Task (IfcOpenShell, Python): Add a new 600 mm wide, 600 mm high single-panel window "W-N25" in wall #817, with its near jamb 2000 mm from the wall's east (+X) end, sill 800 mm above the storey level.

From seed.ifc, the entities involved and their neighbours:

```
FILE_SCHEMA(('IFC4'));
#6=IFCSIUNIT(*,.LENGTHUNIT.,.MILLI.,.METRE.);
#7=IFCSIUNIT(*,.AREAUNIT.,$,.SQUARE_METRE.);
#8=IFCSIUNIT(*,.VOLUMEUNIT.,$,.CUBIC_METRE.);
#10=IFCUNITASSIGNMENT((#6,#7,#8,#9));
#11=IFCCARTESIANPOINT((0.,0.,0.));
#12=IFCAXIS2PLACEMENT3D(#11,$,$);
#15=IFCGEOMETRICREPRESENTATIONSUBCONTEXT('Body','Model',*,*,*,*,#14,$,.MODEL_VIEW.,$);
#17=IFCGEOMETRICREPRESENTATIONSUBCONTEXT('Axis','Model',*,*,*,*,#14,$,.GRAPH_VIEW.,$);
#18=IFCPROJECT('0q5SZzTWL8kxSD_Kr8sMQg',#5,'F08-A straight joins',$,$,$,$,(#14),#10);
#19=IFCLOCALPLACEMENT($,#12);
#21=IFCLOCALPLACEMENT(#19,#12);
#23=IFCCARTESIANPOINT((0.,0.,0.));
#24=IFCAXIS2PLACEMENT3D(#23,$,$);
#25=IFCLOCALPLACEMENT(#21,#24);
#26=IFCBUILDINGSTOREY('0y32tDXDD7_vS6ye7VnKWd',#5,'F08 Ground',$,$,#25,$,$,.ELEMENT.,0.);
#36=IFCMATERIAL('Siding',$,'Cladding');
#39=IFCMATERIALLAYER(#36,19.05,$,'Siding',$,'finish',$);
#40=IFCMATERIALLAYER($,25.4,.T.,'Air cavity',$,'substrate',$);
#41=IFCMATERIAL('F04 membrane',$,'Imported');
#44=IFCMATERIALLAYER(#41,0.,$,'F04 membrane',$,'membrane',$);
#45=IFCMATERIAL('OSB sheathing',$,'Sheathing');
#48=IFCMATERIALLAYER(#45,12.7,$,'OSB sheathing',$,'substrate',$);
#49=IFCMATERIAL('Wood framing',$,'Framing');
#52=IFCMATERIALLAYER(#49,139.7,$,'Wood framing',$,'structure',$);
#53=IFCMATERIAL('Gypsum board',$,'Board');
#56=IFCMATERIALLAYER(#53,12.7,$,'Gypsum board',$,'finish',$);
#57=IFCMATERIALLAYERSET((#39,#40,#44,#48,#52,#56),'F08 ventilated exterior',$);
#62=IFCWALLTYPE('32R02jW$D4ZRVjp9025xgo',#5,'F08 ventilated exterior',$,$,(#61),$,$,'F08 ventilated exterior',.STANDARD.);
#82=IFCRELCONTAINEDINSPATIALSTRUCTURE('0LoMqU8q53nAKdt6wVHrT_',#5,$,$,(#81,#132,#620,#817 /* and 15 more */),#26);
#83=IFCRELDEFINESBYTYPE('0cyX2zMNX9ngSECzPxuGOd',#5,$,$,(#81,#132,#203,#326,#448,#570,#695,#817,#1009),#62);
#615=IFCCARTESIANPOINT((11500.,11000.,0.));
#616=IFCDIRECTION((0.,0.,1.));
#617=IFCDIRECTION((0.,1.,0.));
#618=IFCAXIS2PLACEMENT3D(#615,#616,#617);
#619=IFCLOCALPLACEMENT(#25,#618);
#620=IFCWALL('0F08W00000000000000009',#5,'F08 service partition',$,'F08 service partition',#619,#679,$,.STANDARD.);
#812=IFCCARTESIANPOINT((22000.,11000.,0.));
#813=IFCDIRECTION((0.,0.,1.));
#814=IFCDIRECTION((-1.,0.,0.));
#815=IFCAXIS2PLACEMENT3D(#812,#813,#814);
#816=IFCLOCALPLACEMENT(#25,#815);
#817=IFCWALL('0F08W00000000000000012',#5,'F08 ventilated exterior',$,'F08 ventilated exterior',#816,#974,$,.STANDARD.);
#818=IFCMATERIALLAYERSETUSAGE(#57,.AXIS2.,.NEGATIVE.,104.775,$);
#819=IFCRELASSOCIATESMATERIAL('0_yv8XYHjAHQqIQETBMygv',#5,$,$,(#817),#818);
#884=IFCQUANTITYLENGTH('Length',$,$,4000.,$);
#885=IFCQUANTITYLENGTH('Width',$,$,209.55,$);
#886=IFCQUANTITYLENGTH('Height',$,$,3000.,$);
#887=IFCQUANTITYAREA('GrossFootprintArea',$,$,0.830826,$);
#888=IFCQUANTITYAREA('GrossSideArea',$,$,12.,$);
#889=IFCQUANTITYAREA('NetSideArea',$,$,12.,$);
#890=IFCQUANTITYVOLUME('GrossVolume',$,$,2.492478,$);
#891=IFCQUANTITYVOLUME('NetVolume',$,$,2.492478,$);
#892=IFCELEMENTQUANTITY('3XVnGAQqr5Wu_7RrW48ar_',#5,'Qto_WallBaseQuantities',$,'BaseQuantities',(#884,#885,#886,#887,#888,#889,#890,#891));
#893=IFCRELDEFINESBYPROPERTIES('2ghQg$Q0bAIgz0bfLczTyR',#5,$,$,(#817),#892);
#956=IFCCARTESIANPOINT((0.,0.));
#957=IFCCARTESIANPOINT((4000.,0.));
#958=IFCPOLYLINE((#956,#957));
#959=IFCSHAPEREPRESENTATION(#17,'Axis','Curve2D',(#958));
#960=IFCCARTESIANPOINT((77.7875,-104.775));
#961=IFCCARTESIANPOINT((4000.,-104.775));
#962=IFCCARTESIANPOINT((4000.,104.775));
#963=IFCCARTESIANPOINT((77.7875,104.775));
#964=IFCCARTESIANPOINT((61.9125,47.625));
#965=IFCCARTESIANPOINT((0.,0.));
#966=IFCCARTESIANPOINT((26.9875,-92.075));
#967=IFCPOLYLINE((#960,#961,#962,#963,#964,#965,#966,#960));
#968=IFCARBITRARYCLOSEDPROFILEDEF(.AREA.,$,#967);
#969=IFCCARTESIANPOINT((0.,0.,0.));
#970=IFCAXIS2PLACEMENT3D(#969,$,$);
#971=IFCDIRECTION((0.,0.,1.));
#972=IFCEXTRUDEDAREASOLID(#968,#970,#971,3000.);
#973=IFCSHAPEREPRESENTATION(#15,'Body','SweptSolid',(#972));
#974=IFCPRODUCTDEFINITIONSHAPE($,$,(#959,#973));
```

```python
import numpy as np
import ifcopenshell
import ifcopenshell.api.feature
import ifcopenshell.api.geometry
import ifcopenshell.api.pset
import ifcopenshell.api.root
import ifcopenshell.api.spatial
import ifcopenshell.geom
import ifcopenshell.util.element
import ifcopenshell.util.placement
import ifcopenshell.util.representation
import ifcopenshell.util.shape
import ifcopenshell.util.unit

model = ifcopenshell.open("seed.ifc")
unit_scale = ifcopenshell.util.unit.calculate_unit_scale(model)
area_scale = ifcopenshell.util.unit.calculate_unit_scale(model, "AREAUNIT")
volume_scale = ifcopenshell.util.unit.calculate_unit_scale(model, "VOLUMEUNIT")
settings = ifcopenshell.geom.settings()


def volume(element):
    """Net volume in cubic metres, openings subtracted."""
    shape = ifcopenshell.geom.create_shape(settings, element)
    return ifcopenshell.util.shape.get_volume(shape.geometry)


wall = model.by_guid("0F08W00000000000000012")
storey = ifcopenshell.util.element.get_container(wall, ifc_class="IfcBuildingStorey")
context = ifcopenshell.util.representation.get_context(model, "Model", "Body", "MODEL_VIEW")
before = volume(wall)

width, height, from_end, sill = 0.6, 0.6, 2, 0.8  # metres

# The wall runs along its own X axis, and the end named is its -X end.
wall_shape = ifcopenshell.geom.create_shape(settings, wall)
x, y, z = ifcopenshell.util.shape.get_vertices(wall_shape.geometry).T
start = x.min() + from_end
face, thickness = float(y.min()), float(y.max() - y.min())
wall_matrix = ifcopenshell.util.placement.get_local_placement(wall.ObjectPlacement)
level = ifcopenshell.util.placement.get_local_placement(storey.ObjectPlacement)[2, 3]


def in_wall(x, y):
    """Placement at x, y metres in the wall's axes, at sill height."""
    matrix = wall_matrix.copy()
    matrix[:, 3] = wall_matrix @ np.array([x / unit_scale, y / unit_scale, 0.0, 1.0])
    matrix[2, 3] = level + sill / unit_scale
    return matrix


# Opening: a box that overshoots both wall faces by 50 mm.
opening = ifcopenshell.api.root.create_entity(model, ifc_class="IfcOpeningElement", predefined_type="OPENING")
box = ifcopenshell.api.geometry.add_wall_representation(
    model, context=context, length=width, height=height, thickness=thickness + 0.1
)
ifcopenshell.api.geometry.assign_representation(model, product=opening, representation=box)
ifcopenshell.api.geometry.edit_object_placement(model, product=opening, matrix=in_wall(start, face - 0.05), is_si=False)
ifcopenshell.api.feature.add_feature(model, feature=opening, element=wall)

window = ifcopenshell.api.root.create_entity(model, ifc_class="IfcWindow", name="W-N25", predefined_type="WINDOW")
window.OverallWidth, window.OverallHeight = width / unit_scale, height / unit_scale
window.PartitioningType = "SINGLE_PANEL"
body = ifcopenshell.api.geometry.add_window_representation(
    model,
    context=context,
    overall_width=window.OverallWidth,
    overall_height=window.OverallHeight,
    partition_type="SINGLE_PANEL",
)
ifcopenshell.api.geometry.assign_representation(model, product=window, representation=body)
ifcopenshell.api.spatial.assign_container(model, products=[window], relating_structure=storey)
ifcopenshell.api.feature.add_filling(model, opening=opening, element=window)

# Centre the window in the wall's thickness.
ifcopenshell.api.geometry.edit_object_placement(model, product=window, matrix=in_wall(start, face), is_si=False)
window_shape = ifcopenshell.geom.create_shape(settings, window)
depth = ifcopenshell.util.shape.get_vertices(window_shape.geometry)[:, 1]
offset = face + thickness / 2 - (depth.min() + depth.max()) / 2
ifcopenshell.api.geometry.edit_object_placement(model, product=window, matrix=in_wall(start, offset), is_si=False)

after = volume(wall)

# Update the wall's stored quantities.
qto = model.by_id(ifcopenshell.util.element.get_pset(wall, "Qto_WallBaseQuantities", should_inherit=False)["id"])
ifcopenshell.api.pset.edit_qto(model, qto=qto, properties={
    "NetSideArea": after / thickness / area_scale,
    "NetVolume": after / volume_scale,
})

print(f"wall volume {before:.3f} -> {after:.3f} m3")

model.write("seed_edited.ifc")
```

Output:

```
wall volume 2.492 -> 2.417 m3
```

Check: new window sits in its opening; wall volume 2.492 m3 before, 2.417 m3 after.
